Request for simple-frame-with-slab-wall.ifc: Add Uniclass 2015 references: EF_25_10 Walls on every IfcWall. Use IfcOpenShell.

First a look at what the model holds.

```python
import ifcopenshell

model = ifcopenshell.open("simple-frame-with-slab-wall.ifc")
print(model.schema)
print("classifications:", [c.Name for c in model.by_type("IfcClassification")])
for ifc_class in ("IfcDoor", "IfcRoof", "IfcStair", "IfcWall", "IfcWindow"):
    print(ifc_class, len(model.by_type(ifc_class)))
```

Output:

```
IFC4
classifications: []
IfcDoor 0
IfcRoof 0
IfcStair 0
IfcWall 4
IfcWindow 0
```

```python
import ifcopenshell
import ifcopenshell.api.classification

model = ifcopenshell.open("simple-frame-with-slab-wall.ifc")

system = ifcopenshell.api.classification.add_classification(model, classification="Uniclass 2015")

codes = {
    "IfcWall": ("EF_25_10", "Walls"),
}
for ifc_class, (code, name) in codes.items():
    products = model.by_type(ifc_class)
    ifcopenshell.api.classification.add_reference(
        model, products=products, classification=system, identification=code, name=name
    )
    print(code, len(products))

model.write("simple-frame-with-slab-wall_edited.ifc")
```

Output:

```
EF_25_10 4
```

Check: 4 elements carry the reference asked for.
